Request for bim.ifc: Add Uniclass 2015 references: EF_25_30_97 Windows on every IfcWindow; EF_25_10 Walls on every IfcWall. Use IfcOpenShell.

First a look at what the model holds.

```python
import ifcopenshell

model = ifcopenshell.open("bim.ifc")
print(model.schema)
print("classifications:", [c.Name for c in model.by_type("IfcClassification")])
for ifc_class in ("IfcDoor", "IfcRoof", "IfcStair", "IfcWall", "IfcWindow"):
    print(ifc_class, len(model.by_type(ifc_class)))
```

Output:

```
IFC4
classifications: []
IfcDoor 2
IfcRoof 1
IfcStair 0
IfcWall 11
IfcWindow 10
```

```python
import ifcopenshell
import ifcopenshell.api.classification

model = ifcopenshell.open("bim.ifc")

system = ifcopenshell.api.classification.add_classification(model, classification="Uniclass 2015")

codes = {
    "IfcWindow": ("EF_25_30_97", "Windows"),
    "IfcWall": ("EF_25_10", "Walls"),
}
for ifc_class, (code, name) in codes.items():
    products = model.by_type(ifc_class)
    ifcopenshell.api.classification.add_reference(
        model, products=products, classification=system, identification=code, name=name
    )
    print(code, len(products))

model.write("bim_edited.ifc")
```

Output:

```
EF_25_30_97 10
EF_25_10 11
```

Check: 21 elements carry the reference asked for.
